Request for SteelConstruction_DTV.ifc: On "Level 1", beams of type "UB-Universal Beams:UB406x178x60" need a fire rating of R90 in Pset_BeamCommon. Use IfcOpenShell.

First a look at what the model holds.

```python
import ifcopenshell
import ifcopenshell.util.element

model = ifcopenshell.open("SteelConstruction_DTV.ifc")
print(model.schema)
storey = next(s for s in model.by_type("IfcBuildingStorey") if s.Name == "Level 1")
beams = [e for e in ifcopenshell.util.element.get_decomposition(storey) if e.is_a("IfcBeam")]
seen = {}
for e in beams:
    element_type = ifcopenshell.util.element.get_type(e)
    key = (element_type.Name if element_type != e and element_type else None, ifcopenshell.util.element.get_pset(e, "Pset_BeamCommon", "FireRating"))
    seen[key] = seen.get(key, 0) + 1
for (name, value), count in sorted(seen.items(), key=str):
    print(count, "x", name, "|", value)
```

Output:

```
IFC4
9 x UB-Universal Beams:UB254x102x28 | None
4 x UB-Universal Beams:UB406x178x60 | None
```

```python
import ifcopenshell
import ifcopenshell.api.pset
import ifcopenshell.util.element

model = ifcopenshell.open("SteelConstruction_DTV.ifc")

storey = next(s for s in model.by_type("IfcBuildingStorey") if s.Name == "Level 1")
beams = [e for e in ifcopenshell.util.element.get_decomposition(storey) if e.is_a("IfcBeam")]

count = 0
for e in beams:
    element_type = ifcopenshell.util.element.get_type(e)
    if element_type in (None, e) or element_type.Name != "UB-Universal Beams:UB406x178x60":
        continue
    # add_pset returns the element's existing set when there is one.
    pset = ifcopenshell.api.pset.add_pset(model, product=e, name="Pset_BeamCommon")
    ifcopenshell.api.pset.edit_pset(model, pset=pset, properties={"FireRating": "R90"})
    count += 1

print(count, "beams updated")

model.write("SteelConstruction_DTV_edited.ifc")
```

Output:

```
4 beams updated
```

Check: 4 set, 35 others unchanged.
